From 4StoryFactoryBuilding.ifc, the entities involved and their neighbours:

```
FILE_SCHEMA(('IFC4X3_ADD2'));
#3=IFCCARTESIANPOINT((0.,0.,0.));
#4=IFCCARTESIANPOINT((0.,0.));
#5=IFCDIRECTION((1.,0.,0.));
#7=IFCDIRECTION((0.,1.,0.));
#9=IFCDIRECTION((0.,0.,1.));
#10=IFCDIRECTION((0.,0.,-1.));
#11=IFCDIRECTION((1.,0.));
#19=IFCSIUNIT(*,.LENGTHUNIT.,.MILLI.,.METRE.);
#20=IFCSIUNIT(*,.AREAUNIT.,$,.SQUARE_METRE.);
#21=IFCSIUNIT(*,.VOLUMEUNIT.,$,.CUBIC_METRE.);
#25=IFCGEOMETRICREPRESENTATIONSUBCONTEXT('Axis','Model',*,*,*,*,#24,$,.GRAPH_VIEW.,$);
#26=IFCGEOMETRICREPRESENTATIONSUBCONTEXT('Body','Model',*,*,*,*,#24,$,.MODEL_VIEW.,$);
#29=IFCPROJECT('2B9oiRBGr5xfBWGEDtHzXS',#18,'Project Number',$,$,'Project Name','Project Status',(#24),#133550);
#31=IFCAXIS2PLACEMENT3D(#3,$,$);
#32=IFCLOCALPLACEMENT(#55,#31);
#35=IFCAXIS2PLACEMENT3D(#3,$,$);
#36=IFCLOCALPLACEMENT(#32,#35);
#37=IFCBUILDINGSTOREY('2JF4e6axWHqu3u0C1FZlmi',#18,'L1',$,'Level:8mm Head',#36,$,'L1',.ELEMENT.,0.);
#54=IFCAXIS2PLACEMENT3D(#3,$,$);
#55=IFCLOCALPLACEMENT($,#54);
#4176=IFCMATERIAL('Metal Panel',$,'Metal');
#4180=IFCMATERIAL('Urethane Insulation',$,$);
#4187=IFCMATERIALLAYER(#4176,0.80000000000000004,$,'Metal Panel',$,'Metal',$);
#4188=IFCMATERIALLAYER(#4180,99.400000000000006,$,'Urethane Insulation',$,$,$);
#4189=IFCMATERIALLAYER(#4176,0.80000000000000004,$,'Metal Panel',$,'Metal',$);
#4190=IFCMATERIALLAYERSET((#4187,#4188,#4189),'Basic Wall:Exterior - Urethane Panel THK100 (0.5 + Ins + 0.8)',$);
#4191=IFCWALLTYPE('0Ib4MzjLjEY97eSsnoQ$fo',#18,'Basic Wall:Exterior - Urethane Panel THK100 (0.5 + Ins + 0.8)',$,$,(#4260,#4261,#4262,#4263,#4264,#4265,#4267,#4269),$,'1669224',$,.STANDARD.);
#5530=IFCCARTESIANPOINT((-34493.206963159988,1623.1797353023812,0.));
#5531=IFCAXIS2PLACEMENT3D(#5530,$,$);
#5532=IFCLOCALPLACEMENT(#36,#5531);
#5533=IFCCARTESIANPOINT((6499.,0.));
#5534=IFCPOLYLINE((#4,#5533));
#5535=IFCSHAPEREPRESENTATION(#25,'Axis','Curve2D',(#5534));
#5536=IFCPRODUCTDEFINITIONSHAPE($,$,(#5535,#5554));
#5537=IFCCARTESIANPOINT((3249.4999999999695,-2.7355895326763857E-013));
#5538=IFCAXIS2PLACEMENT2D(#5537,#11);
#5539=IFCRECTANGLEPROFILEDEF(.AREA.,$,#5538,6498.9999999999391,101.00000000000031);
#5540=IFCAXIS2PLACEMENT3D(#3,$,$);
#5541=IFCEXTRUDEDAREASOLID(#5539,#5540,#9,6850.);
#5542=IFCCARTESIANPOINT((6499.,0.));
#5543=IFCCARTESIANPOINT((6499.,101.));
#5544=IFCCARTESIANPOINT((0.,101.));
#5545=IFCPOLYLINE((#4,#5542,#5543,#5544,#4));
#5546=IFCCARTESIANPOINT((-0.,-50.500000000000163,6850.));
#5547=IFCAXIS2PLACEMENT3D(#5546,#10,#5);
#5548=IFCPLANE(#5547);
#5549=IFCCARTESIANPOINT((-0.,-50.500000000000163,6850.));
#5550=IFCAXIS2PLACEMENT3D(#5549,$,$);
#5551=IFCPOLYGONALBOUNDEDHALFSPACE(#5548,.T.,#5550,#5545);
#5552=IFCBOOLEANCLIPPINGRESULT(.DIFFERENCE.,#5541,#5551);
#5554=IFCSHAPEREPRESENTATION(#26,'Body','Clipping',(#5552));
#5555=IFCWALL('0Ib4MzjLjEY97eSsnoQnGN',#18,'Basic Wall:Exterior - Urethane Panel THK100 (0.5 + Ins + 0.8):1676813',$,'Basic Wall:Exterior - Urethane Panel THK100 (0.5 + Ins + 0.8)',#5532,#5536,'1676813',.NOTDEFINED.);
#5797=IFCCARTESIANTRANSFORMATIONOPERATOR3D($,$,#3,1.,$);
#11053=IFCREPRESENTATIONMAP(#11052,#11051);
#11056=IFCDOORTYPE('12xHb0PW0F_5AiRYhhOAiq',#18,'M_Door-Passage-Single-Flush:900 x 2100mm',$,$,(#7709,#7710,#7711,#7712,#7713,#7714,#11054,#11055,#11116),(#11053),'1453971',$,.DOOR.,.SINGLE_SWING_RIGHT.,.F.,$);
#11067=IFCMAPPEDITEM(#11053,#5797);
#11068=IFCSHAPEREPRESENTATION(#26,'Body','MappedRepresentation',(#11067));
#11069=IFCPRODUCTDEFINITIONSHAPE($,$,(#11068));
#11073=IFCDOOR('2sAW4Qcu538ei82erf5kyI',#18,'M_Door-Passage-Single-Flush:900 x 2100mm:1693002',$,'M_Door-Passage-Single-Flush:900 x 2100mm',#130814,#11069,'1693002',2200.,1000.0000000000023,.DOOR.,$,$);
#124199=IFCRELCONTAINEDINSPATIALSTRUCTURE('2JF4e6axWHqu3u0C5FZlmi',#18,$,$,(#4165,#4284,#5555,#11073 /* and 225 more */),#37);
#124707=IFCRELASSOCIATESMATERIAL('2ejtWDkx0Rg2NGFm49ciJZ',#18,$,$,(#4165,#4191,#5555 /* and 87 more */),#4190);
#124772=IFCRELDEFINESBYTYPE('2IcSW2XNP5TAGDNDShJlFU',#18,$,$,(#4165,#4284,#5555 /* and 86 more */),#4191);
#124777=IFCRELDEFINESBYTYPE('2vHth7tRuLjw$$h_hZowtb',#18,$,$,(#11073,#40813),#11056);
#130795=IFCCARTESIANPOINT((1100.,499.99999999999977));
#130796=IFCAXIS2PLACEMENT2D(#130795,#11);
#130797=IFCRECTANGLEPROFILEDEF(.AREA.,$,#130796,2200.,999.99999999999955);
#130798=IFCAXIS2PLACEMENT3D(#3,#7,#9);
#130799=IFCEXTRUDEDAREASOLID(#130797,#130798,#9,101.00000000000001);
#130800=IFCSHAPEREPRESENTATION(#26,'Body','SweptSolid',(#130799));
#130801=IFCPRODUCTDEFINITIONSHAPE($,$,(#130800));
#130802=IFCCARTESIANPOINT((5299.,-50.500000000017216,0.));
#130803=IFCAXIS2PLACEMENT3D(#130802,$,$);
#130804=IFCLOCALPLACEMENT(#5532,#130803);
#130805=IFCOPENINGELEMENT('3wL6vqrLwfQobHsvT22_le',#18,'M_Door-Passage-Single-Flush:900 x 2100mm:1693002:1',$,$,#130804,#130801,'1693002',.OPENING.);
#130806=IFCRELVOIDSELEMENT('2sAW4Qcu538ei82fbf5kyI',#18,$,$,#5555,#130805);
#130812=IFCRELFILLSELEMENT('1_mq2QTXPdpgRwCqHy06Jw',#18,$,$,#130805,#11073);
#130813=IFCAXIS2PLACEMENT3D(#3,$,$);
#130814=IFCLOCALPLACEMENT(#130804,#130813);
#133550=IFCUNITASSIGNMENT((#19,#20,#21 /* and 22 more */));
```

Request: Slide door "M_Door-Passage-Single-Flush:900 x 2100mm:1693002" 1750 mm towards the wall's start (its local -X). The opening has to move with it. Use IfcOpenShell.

```python
import ifcopenshell
import ifcopenshell.api.geometry
import ifcopenshell.util.placement

model = ifcopenshell.open("4StoryFactoryBuilding.ifc")

door = model.by_guid("2sAW4Qcu538ei82erf5kyI")
opening = door.FillsVoids[0].RelatingOpeningElement
wall = opening.VoidsElements[0].RelatingBuildingElement

wall_matrix = ifcopenshell.util.placement.get_local_placement(wall.ObjectPlacement)
shift = wall_matrix[:3, 0] * -1750.0
before = ifcopenshell.util.placement.get_local_placement(door.ObjectPlacement)[:3, 3].copy()

# The door is placed relative to its opening, so it follows when the opening moves.
matrix = ifcopenshell.util.placement.get_local_placement(opening.ObjectPlacement)
matrix[:3, 3] += shift
ifcopenshell.api.geometry.edit_object_placement(
    model, product=opening, matrix=matrix, is_si=False, should_transform_children=True
)

after = ifcopenshell.util.placement.get_local_placement(door.ObjectPlacement)[:3, 3]
print("door moved by", (after - before).round(3) + 0.0)

model.write("4StoryFactoryBuilding_rev.ifc")
```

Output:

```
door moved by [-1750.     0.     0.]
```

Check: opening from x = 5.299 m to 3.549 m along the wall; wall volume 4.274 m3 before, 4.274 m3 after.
